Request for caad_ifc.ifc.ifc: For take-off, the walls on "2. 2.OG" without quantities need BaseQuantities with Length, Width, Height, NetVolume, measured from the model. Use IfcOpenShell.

First a look at what the model holds.

```python
import ifcopenshell
import ifcopenshell.util.element
import ifcopenshell.util.unit

model = ifcopenshell.open("caad_ifc.ifc.ifc")
print(model.schema)
for unit_type in ("LENGTHUNIT", "AREAUNIT", "VOLUMEUNIT"):
    print(unit_type, ifcopenshell.util.unit.calculate_unit_scale(model, unit_type))
storey = next(s for s in model.by_type("IfcBuildingStorey") if s.Name == "2. 2.OG")
walls = [e for e in ifcopenshell.util.element.get_decomposition(storey) if e.is_a("IfcWall")]
for e in sorted(walls, key=lambda e: e.id()):
    print(e.id(), e.is_a(), e.Name, list(ifcopenshell.util.element.get_psets(e, qtos_only=True)), sep=" | ")
```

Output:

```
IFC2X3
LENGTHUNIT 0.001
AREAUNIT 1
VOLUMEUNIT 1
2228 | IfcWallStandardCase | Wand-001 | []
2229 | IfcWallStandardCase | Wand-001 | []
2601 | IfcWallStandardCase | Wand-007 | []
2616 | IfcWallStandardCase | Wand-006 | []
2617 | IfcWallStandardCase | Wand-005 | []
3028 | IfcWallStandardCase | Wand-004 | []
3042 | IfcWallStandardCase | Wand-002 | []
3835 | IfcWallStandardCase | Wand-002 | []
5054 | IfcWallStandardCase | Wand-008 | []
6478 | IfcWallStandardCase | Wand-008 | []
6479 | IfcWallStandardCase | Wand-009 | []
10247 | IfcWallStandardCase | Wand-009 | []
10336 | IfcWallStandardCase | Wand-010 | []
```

```python
import ifcopenshell
import ifcopenshell.api.pset
import ifcopenshell.geom
import ifcopenshell.util.element
import ifcopenshell.util.shape
import ifcopenshell.util.unit

model = ifcopenshell.open("caad_ifc.ifc.ifc")
unit_scale = ifcopenshell.util.unit.calculate_unit_scale(model)
volume_scale = ifcopenshell.util.unit.calculate_unit_scale(model, "VOLUMEUNIT")
settings = ifcopenshell.geom.settings()

storey = next(s for s in model.by_type("IfcBuildingStorey") if s.Name == "2. 2.OG")
walls = [e for e in ifcopenshell.util.element.get_decomposition(storey) if e.is_a("IfcWall")]

for e in sorted(walls, key=lambda e: e.id()):
    if ifcopenshell.util.element.get_psets(e, qtos_only=True, should_inherit=False):
        continue
    # Geometry comes back in metres, in the element's own axes.
    shape = ifcopenshell.geom.create_shape(settings, e)
    values = {
        "Length": ifcopenshell.util.shape.get_x(shape.geometry) / unit_scale,
        "Width": ifcopenshell.util.shape.get_y(shape.geometry) / unit_scale,
        "Height": ifcopenshell.util.shape.get_z(shape.geometry) / unit_scale,
        "NetVolume": ifcopenshell.util.shape.get_volume(shape.geometry) / volume_scale,
    }
    qto = ifcopenshell.api.pset.add_qto(model, product=e, name="BaseQuantities")
    ifcopenshell.api.pset.edit_qto(model, qto=qto, properties=values)
    print(e.id(), {k: round(v, 3) for k, v in values.items()})

model.write("caad_ifc.ifc_v2.ifc")
```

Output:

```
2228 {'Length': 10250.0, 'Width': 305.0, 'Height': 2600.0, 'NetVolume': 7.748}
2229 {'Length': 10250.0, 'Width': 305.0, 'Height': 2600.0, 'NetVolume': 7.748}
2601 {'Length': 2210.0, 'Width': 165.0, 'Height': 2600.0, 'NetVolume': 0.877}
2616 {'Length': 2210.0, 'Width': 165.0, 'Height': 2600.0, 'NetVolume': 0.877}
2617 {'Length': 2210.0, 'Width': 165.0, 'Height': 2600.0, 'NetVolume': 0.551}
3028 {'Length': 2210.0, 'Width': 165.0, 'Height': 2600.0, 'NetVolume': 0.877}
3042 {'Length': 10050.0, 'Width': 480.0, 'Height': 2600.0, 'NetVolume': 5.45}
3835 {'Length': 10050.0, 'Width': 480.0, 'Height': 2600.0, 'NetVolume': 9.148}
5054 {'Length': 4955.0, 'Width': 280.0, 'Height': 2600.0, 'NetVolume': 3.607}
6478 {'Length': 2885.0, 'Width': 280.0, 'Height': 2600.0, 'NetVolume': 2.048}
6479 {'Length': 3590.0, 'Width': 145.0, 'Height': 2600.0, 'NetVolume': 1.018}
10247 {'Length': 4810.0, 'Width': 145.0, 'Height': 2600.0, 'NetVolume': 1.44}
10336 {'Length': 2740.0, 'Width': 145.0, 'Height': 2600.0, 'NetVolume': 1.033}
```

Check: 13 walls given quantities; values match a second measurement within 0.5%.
